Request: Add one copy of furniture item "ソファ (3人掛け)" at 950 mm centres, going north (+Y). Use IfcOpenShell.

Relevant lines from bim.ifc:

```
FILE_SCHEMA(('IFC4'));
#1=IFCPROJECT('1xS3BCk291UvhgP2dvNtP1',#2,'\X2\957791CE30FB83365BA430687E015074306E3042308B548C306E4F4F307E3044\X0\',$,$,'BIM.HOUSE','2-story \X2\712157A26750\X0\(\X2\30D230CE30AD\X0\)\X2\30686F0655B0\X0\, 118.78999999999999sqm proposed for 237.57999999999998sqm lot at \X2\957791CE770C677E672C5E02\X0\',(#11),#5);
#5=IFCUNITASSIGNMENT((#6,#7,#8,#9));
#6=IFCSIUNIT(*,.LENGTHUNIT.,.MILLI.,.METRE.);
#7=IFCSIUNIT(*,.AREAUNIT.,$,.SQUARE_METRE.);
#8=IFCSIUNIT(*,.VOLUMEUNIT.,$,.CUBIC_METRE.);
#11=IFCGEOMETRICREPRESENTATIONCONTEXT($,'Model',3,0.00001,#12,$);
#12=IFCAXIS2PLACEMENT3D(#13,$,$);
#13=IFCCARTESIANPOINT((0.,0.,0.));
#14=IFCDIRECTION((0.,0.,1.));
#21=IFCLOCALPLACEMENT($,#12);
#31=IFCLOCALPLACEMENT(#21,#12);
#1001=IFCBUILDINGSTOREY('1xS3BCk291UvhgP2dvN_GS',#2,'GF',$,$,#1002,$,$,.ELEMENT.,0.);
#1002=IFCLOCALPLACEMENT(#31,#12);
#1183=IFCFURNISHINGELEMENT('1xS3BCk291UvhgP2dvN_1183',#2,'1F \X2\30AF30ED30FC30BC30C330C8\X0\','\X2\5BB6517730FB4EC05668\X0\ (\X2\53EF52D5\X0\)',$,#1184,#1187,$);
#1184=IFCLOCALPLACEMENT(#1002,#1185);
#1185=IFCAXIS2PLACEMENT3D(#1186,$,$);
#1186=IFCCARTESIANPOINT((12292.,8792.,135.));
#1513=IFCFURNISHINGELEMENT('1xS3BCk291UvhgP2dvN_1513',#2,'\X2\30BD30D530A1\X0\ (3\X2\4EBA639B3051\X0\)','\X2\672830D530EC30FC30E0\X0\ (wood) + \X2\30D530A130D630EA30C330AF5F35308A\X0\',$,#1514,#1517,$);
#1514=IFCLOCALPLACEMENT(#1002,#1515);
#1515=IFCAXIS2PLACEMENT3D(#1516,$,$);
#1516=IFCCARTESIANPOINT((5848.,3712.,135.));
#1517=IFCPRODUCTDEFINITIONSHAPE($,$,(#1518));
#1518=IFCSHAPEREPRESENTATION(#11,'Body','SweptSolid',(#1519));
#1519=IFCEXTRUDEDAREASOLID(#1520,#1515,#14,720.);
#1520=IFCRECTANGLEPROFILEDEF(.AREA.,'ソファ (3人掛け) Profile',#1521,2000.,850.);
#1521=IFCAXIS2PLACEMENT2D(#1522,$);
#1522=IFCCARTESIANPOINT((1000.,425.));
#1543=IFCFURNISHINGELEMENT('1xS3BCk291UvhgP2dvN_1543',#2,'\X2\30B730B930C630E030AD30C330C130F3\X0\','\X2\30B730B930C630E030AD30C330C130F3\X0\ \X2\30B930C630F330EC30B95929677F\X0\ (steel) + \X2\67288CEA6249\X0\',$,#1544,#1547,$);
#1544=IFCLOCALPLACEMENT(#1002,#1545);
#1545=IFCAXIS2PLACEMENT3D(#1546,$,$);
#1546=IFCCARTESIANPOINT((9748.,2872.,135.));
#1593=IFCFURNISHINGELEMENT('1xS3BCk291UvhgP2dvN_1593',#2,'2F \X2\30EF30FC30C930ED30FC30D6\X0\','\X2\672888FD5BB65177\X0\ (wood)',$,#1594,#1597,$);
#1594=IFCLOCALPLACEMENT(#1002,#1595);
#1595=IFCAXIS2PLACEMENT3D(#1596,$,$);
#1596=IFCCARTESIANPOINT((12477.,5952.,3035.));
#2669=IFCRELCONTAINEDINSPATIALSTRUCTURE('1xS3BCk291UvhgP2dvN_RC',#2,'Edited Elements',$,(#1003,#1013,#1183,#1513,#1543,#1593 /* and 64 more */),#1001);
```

```python
import numpy as np
import ifcopenshell
import ifcopenshell.api.geometry
import ifcopenshell.api.root
import ifcopenshell.util.element
import ifcopenshell.util.placement
import ifcopenshell.util.unit

model = ifcopenshell.open("bim.ifc")
unit_scale = ifcopenshell.util.unit.calculate_unit_scale(model)


def reuse_history(source, copy):
    """copy_class also copies each property set's owner history, people and application; keep the originals."""
    for rel in copy.IsDefinedBy:
        if rel.is_a("IfcRelDefinesByProperties") and (history := rel.RelatingPropertyDefinition.OwnerHistory):
            rel.RelatingPropertyDefinition.OwnerHistory = source.OwnerHistory
            ifcopenshell.util.element.remove_deep2(model, history)


source = model.by_guid("1xS3BCk291UvhgP2dvN_1513")
base = ifcopenshell.util.placement.get_local_placement(source.ObjectPlacement)
step = np.array([0.0, 1.0, 0.0]) * 0.95 / unit_scale

for i in range(1, 2):
    copy = ifcopenshell.api.root.copy_class(model, product=source)
    copy.Representation = ifcopenshell.util.element.copy_deep(
        model, source.Representation, exclude=["IfcGeometricRepresentationContext", "IfcRepresentationMap"]
    )
    reuse_history(source, copy)
    matrix = base.copy()
    matrix[:3, 3] += i * step
    print("added at", matrix[:3, 3].round(3) + 0.0)
    ifcopenshell.api.geometry.edit_object_placement(model, product=copy, matrix=matrix, is_si=False)

model.write("bim-out.ifc")
```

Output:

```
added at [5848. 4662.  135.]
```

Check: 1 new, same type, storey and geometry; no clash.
